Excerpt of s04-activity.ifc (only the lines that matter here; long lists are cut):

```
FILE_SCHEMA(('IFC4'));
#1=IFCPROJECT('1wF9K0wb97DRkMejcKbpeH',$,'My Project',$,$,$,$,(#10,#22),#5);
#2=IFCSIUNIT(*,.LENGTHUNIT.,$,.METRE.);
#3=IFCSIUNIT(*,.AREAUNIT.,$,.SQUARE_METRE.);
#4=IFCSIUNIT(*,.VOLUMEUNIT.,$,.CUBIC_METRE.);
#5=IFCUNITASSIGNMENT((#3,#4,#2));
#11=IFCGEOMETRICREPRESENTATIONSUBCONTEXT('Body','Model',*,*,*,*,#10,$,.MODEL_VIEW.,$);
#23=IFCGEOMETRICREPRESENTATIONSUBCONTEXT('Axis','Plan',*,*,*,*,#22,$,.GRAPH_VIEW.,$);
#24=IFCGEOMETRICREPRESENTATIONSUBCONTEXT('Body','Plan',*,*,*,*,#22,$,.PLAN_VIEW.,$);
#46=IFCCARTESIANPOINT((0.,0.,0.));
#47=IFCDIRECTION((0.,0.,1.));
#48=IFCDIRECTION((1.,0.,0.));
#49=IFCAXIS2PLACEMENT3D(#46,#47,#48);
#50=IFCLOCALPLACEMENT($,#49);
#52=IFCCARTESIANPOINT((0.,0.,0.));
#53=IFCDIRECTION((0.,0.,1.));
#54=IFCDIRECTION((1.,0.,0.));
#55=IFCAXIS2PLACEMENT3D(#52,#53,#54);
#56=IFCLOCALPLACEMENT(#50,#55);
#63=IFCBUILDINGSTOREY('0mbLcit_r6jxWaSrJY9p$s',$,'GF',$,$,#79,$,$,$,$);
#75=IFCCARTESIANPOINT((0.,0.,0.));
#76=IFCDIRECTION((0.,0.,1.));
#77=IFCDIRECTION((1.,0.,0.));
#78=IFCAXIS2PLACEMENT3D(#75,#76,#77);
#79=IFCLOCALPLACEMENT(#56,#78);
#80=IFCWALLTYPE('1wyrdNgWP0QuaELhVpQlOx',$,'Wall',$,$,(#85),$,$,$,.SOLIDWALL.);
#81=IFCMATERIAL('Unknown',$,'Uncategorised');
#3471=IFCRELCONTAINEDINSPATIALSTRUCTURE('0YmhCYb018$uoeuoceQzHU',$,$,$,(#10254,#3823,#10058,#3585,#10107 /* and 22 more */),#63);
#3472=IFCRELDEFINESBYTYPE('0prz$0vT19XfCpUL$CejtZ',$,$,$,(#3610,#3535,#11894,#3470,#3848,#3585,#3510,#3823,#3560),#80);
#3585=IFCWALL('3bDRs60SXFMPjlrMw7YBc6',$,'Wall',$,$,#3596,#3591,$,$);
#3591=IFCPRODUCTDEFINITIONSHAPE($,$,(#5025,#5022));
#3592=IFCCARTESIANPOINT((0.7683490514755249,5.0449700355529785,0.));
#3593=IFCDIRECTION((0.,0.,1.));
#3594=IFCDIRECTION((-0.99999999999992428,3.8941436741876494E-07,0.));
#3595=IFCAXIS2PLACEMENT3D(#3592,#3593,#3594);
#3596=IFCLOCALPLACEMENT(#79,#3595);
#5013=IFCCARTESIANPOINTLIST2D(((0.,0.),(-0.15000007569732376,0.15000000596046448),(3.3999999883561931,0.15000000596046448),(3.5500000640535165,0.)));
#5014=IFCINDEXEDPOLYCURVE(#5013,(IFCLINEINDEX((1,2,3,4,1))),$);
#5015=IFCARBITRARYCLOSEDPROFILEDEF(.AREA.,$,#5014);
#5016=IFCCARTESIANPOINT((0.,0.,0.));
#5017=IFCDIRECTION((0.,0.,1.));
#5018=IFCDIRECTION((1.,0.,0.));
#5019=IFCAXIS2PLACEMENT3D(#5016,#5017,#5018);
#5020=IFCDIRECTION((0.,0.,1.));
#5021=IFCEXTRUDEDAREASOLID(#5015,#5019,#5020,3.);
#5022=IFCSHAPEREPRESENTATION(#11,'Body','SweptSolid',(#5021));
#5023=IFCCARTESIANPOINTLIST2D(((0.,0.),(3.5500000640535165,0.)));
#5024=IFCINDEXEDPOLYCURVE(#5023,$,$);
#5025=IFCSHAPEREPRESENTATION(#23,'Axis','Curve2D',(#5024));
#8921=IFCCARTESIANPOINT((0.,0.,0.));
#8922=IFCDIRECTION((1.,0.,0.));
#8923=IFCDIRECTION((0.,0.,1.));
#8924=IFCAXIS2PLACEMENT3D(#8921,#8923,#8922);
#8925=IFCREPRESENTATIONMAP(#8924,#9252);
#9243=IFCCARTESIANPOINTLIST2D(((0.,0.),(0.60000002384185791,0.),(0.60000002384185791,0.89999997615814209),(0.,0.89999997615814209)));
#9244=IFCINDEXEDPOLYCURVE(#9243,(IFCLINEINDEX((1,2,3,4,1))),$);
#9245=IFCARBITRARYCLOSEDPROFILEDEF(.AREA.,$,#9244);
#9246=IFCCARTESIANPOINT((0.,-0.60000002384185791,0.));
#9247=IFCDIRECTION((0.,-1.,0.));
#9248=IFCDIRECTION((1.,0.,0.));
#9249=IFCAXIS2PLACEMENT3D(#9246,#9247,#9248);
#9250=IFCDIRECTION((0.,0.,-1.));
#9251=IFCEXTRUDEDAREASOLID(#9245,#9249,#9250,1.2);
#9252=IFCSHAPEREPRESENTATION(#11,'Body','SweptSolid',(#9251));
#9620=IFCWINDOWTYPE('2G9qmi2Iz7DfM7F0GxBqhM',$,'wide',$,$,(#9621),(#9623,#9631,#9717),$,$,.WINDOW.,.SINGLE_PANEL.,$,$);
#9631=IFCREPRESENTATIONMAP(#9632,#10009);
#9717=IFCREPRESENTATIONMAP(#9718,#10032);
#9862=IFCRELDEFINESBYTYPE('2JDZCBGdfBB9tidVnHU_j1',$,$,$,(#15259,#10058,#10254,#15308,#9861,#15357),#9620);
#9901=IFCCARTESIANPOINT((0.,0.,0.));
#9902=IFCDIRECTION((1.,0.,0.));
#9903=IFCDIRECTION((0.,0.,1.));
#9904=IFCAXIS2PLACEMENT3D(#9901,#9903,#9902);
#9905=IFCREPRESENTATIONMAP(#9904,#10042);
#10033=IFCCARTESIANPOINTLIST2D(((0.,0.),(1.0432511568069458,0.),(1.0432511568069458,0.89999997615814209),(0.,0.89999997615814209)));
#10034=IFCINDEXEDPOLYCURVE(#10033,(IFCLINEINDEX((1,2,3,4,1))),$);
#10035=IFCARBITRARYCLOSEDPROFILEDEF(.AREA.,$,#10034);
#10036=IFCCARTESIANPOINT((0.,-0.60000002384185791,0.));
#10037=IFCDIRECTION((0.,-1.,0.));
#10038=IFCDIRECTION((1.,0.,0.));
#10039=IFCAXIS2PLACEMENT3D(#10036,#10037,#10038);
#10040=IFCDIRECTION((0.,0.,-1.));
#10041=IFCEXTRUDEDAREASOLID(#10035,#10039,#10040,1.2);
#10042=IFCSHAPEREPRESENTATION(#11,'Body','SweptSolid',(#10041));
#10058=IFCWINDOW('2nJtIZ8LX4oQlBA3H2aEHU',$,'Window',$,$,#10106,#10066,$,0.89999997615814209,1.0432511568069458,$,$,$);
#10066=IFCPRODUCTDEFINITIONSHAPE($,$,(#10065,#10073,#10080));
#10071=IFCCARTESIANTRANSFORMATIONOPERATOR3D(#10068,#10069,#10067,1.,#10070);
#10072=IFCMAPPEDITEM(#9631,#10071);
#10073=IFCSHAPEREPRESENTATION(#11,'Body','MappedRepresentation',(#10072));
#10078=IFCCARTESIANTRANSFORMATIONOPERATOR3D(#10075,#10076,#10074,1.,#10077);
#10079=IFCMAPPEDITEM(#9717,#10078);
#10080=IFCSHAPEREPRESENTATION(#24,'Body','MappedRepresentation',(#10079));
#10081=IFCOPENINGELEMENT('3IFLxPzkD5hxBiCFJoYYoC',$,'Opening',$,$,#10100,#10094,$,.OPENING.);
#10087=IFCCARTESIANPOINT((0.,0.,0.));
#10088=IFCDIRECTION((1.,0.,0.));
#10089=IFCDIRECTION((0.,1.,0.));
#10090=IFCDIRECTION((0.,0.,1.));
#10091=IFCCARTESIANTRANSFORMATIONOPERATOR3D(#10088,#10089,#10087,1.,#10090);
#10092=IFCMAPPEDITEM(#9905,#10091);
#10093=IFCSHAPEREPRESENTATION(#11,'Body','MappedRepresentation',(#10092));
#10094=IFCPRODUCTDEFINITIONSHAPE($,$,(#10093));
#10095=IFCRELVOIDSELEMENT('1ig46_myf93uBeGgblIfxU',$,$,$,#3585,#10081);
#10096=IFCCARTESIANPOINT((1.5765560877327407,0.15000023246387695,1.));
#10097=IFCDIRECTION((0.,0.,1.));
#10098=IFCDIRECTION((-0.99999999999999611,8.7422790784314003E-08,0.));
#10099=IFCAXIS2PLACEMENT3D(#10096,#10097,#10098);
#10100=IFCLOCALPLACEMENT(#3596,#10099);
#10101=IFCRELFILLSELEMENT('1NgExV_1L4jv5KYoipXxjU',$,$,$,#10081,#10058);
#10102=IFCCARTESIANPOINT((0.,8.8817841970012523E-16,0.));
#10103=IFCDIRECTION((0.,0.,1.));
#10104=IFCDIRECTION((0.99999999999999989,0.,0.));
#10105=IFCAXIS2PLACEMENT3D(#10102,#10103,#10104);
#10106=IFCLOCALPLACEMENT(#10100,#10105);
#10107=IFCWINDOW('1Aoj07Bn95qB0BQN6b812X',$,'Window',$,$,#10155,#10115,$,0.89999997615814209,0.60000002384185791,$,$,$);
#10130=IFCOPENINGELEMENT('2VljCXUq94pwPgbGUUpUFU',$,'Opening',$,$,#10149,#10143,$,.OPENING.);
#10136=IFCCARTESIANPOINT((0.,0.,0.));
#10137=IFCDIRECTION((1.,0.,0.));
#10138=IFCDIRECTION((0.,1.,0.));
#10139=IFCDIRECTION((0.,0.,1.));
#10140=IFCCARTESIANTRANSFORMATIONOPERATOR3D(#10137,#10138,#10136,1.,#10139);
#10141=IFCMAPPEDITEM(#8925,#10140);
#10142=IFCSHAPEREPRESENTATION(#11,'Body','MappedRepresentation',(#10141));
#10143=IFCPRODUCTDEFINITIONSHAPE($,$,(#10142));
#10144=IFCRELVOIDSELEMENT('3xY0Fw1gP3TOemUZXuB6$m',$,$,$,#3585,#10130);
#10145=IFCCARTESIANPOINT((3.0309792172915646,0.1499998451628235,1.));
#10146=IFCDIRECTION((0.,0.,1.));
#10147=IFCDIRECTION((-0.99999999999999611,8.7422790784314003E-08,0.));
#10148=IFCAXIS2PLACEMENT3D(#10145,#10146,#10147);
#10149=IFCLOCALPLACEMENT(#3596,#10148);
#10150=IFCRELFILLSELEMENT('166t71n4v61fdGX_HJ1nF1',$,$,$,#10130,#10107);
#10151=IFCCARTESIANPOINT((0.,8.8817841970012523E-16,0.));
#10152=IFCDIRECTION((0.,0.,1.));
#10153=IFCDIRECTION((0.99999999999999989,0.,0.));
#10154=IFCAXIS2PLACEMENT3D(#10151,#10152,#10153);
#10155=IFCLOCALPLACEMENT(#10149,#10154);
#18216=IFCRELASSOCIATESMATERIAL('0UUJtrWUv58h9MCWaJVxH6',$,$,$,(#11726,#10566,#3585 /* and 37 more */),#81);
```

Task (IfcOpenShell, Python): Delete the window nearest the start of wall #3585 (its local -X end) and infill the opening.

```python
import ifcopenshell
import ifcopenshell.api.feature
import ifcopenshell.api.root
import ifcopenshell.geom
import ifcopenshell.util.shape

model = ifcopenshell.open("s04-activity.ifc")
settings = ifcopenshell.geom.settings()


def volume(element):
    """Net volume in cubic metres, openings subtracted."""
    shape = ifcopenshell.geom.create_shape(settings, element)
    return ifcopenshell.util.shape.get_volume(shape.geometry)


window = model.by_guid("2nJtIZ8LX4oQlBA3H2aEHU")
opening = window.FillsVoids[0].RelatingOpeningElement
wall = opening.VoidsElements[0].RelatingBuildingElement
before = volume(wall)

ifcopenshell.api.root.remove_product(model, product=window)
ifcopenshell.api.feature.remove_feature(model, feature=opening)

after = volume(wall)

print(f"wall volume {before:.3f} -> {after:.3f} m3")

model.write("s04-activity-out.ifc")
```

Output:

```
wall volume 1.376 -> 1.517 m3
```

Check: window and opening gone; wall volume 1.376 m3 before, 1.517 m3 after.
